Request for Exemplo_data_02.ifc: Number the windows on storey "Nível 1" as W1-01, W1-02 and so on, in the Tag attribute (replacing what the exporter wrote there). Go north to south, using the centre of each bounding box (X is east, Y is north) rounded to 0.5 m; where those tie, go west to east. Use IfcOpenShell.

First a look at what the model holds.

```python
import ifcopenshell
import ifcopenshell.util.element
import ifcopenshell.util.placement

model = ifcopenshell.open("Exemplo_data_02.ifc")
print(model.schema)
storey = next(s for s in model.by_type("IfcBuildingStorey") if s.Name == "Nível 1")
windows = [e for e in ifcopenshell.util.element.get_decomposition(storey) if e.is_a("IfcWindow")]
for e in sorted(windows, key=lambda e: e.id()):
    origin = ifcopenshell.util.placement.get_local_placement(e.ObjectPlacement)[:3, 3]
    print(e.id(), e.Tag, e.Name, origin.round(2) + 0.0, sep=" | ")
```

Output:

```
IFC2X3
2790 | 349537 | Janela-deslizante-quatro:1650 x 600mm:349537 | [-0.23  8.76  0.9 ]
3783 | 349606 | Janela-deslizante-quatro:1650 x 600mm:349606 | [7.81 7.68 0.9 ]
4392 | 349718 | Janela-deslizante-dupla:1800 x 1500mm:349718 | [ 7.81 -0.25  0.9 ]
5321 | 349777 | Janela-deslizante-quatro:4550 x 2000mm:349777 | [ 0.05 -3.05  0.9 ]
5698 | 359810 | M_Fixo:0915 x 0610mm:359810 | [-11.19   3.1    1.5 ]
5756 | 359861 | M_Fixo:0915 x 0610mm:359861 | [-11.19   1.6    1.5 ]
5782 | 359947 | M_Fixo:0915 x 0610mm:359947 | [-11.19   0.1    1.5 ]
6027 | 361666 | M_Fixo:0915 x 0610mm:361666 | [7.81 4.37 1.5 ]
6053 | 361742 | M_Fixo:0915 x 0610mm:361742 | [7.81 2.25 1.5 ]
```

```python
import ifcopenshell
import ifcopenshell.geom
import ifcopenshell.util.element
import ifcopenshell.util.shape

model = ifcopenshell.open("Exemplo_data_02.ifc")
settings = ifcopenshell.geom.settings()
settings.set("use-world-coords", True)


def centre(element):
    shape = ifcopenshell.geom.create_shape(settings, element)
    return ifcopenshell.util.shape.get_bbox_centroid(shape.geometry)


storey = next(s for s in model.by_type("IfcBuildingStorey") if s.Name == "Nível 1")
windows = [e for e in ifcopenshell.util.element.get_decomposition(storey) if e.is_a("IfcWindow")]

# Insertion points can sit at a corner or the storey origin, so sort by the geometry (in metres).
centres = {e: centre(e) for e in windows}
windows.sort(key=lambda e: (-round(centres[e][1] / 0.5), centres[e][0]))

for i, e in enumerate(windows, start=1):
    number = f"W1-{i:02d}"
    e.Tag = number
    print(e.id(), number)

model.write("Exemplo_data_02-out.ifc")
```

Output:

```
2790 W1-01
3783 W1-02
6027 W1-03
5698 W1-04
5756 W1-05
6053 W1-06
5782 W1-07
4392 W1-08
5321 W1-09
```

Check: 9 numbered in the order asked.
